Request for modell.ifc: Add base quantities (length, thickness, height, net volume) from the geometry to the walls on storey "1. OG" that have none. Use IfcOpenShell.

First a look at what the model holds.

```python
import ifcopenshell
import ifcopenshell.util.element
import ifcopenshell.util.unit

model = ifcopenshell.open("modell.ifc")
print(model.schema)
for unit_type in ("LENGTHUNIT", "AREAUNIT", "VOLUMEUNIT"):
    print(unit_type, ifcopenshell.util.unit.calculate_unit_scale(model, unit_type))
storey = next(s for s in model.by_type("IfcBuildingStorey") if s.Name == "1. OG")
walls = [e for e in ifcopenshell.util.element.get_decomposition(storey) if e.is_a("IfcWall")]
for e in sorted(walls, key=lambda e: e.id()):
    print(e.id(), e.is_a(), e.Name, list(ifcopenshell.util.element.get_psets(e, qtos_only=True)), sep=" | ")
```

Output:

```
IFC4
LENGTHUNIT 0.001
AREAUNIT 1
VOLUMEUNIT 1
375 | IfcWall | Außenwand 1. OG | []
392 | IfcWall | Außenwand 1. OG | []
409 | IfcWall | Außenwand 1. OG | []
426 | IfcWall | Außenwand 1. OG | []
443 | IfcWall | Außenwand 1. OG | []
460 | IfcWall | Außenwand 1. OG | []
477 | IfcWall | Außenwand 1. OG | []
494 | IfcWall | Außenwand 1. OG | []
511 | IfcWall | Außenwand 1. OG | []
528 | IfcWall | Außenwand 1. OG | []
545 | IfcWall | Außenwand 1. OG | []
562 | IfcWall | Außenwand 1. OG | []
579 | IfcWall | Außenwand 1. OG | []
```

```python
import ifcopenshell
import ifcopenshell.api.pset
import ifcopenshell.geom
import ifcopenshell.util.element
import ifcopenshell.util.shape
import ifcopenshell.util.unit

model = ifcopenshell.open("modell.ifc")
unit_scale = ifcopenshell.util.unit.calculate_unit_scale(model)
volume_scale = ifcopenshell.util.unit.calculate_unit_scale(model, "VOLUMEUNIT")
settings = ifcopenshell.geom.settings()

storey = next(s for s in model.by_type("IfcBuildingStorey") if s.Name == "1. OG")
walls = [e for e in ifcopenshell.util.element.get_decomposition(storey) if e.is_a("IfcWall")]

for e in sorted(walls, key=lambda e: e.id()):
    if ifcopenshell.util.element.get_psets(e, qtos_only=True, should_inherit=False):
        continue
    # Geometry comes back in metres, in the element's own axes.
    shape = ifcopenshell.geom.create_shape(settings, e)
    values = {
        "Length": ifcopenshell.util.shape.get_x(shape.geometry) / unit_scale,
        "Width": ifcopenshell.util.shape.get_y(shape.geometry) / unit_scale,
        "Height": ifcopenshell.util.shape.get_z(shape.geometry) / unit_scale,
        "NetVolume": ifcopenshell.util.shape.get_volume(shape.geometry) / volume_scale,
    }
    qto = ifcopenshell.api.pset.add_qto(model, product=e, name="Qto_WallBaseQuantities")
    ifcopenshell.api.pset.edit_qto(model, qto=qto, properties=values)
    print(e.id(), {k: round(v, 3) for k, v in values.items()})

model.write("modell_edited.ifc")
```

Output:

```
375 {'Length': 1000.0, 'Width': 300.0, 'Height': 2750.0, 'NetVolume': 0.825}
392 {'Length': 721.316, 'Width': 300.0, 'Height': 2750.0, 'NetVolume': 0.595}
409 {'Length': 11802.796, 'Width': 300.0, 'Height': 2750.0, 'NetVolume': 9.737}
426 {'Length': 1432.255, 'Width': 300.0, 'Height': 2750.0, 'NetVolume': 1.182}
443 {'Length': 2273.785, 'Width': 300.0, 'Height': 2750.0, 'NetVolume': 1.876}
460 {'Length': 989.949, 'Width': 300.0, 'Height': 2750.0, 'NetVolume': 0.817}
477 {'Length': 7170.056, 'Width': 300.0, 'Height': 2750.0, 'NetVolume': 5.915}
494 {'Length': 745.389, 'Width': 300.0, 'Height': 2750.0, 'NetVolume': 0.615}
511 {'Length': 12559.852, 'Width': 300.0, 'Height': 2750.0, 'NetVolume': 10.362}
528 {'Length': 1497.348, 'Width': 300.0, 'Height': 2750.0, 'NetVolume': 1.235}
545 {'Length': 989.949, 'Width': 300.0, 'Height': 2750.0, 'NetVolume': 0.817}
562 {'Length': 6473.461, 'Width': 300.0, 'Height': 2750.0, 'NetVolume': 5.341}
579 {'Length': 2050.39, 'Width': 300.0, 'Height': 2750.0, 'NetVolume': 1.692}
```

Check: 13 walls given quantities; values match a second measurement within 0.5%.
